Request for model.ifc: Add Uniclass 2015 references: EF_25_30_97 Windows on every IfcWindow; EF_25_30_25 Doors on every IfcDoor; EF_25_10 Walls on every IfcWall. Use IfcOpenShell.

First a look at what the model holds.

```python
import ifcopenshell

model = ifcopenshell.open("model.ifc")
print(model.schema)
print("classifications:", [c.Name for c in model.by_type("IfcClassification")])
for ifc_class in ("IfcDoor", "IfcRoof", "IfcStair", "IfcWall", "IfcWindow"):
    print(ifc_class, len(model.by_type(ifc_class)))
```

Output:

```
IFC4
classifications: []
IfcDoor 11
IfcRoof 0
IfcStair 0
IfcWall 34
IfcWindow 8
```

```python
import ifcopenshell
import ifcopenshell.api.classification

model = ifcopenshell.open("model.ifc")

system = ifcopenshell.api.classification.add_classification(model, classification="Uniclass 2015")

codes = {
    "IfcWindow": ("EF_25_30_97", "Windows"),
    "IfcDoor": ("EF_25_30_25", "Doors"),
    "IfcWall": ("EF_25_10", "Walls"),
}
for ifc_class, (code, name) in codes.items():
    products = model.by_type(ifc_class)
    ifcopenshell.api.classification.add_reference(
        model, products=products, classification=system, identification=code, name=name
    )
    print(code, len(products))

model.write("model_v2.ifc")
```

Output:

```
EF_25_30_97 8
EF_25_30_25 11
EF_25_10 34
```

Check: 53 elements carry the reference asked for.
